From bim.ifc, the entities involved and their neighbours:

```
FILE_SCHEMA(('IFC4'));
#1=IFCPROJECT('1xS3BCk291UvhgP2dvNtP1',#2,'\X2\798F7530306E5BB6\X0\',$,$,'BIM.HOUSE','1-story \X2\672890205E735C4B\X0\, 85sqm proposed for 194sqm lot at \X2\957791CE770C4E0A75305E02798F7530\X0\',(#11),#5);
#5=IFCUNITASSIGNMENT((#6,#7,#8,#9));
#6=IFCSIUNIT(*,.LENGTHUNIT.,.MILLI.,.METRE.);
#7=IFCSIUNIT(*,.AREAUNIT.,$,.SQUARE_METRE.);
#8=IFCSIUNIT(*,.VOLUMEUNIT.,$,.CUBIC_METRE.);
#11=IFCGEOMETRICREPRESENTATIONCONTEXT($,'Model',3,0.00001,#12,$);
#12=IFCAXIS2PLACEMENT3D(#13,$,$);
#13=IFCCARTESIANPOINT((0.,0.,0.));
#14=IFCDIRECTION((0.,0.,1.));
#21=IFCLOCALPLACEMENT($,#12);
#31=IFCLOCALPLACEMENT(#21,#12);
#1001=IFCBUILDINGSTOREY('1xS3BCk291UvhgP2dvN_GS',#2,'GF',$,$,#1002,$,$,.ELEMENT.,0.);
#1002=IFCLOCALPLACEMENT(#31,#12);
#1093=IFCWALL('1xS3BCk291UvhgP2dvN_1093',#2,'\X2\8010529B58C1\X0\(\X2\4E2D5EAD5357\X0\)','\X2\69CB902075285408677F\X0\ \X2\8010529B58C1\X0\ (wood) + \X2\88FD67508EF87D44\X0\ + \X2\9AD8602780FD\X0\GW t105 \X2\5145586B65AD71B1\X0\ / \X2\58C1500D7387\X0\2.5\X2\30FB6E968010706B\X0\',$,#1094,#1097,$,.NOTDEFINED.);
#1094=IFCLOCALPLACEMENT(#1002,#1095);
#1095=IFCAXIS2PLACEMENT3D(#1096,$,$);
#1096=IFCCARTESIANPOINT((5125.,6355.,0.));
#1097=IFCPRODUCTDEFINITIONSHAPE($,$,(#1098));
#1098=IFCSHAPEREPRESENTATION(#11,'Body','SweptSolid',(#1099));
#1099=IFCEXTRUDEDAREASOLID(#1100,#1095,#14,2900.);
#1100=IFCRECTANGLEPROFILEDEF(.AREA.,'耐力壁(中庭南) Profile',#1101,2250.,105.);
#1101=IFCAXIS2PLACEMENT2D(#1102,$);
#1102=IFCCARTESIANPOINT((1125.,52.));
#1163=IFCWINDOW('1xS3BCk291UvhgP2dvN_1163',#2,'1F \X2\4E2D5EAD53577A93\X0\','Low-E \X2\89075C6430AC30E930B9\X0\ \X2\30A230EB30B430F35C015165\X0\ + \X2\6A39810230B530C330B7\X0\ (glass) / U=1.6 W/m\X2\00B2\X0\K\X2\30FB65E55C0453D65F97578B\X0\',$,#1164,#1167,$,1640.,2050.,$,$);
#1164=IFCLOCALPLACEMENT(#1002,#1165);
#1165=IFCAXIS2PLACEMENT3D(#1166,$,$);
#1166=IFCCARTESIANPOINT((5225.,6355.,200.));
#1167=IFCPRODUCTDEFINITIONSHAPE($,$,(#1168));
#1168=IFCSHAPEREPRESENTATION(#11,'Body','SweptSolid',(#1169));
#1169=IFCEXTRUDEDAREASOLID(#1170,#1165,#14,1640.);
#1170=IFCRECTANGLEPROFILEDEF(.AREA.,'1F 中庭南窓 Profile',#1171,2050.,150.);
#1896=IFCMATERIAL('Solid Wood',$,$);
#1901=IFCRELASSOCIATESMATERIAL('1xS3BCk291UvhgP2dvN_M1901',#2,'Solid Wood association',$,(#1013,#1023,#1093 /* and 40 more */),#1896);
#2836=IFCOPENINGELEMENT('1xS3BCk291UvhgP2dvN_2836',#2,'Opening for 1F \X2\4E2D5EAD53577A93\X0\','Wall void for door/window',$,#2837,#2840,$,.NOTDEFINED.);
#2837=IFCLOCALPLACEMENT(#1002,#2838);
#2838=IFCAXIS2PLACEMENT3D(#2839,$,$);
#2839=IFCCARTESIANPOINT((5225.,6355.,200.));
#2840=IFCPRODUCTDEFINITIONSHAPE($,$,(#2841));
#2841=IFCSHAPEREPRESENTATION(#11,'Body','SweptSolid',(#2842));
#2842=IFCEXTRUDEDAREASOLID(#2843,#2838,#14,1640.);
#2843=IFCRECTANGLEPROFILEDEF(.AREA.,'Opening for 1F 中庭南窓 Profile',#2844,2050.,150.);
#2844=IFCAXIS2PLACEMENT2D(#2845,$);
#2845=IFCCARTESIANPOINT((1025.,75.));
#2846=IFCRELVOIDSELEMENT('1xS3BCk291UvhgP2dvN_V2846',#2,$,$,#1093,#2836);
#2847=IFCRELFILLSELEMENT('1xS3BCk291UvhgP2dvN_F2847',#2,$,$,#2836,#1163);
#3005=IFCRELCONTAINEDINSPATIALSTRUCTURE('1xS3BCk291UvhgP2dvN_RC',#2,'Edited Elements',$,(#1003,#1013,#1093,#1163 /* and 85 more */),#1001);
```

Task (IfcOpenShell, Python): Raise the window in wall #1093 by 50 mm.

```python
import numpy as np
import ifcopenshell
import ifcopenshell.api.geometry
import ifcopenshell.util.placement
import ifcopenshell.util.unit

model = ifcopenshell.open("bim.ifc")
unit_scale = ifcopenshell.util.unit.calculate_unit_scale(model)

window = model.by_guid("1xS3BCk291UvhgP2dvN_1163")
opening = window.FillsVoids[0].RelatingOpeningElement
dz = 0.05 / unit_scale

shift = np.array([0.0, 0.0, dz])
# The window is not placed relative to its opening, so move both.
for product in (opening, window):
    matrix = ifcopenshell.util.placement.get_local_placement(product.ObjectPlacement)
    matrix[:3, 3] += shift
    ifcopenshell.api.geometry.edit_object_placement(model, product=product, matrix=matrix, is_si=False)

print(f"moved by {dz * unit_scale:+.3f} m")

model.write("bim_rev.ifc")
```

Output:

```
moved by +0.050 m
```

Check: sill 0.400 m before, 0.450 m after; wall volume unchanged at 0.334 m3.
